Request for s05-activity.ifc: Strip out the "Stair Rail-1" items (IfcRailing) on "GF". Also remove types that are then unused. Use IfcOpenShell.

First a look at what the model holds.

```python
import ifcopenshell
import ifcopenshell.util.element

model = ifcopenshell.open("s05-activity.ifc")
print(model.schema)
storey = next(s for s in model.by_type("IfcBuildingStorey") if s.Name == "GF")
railings = [e for e in ifcopenshell.util.element.get_decomposition(storey) if e.is_a("IfcRailing")]
seen = {}
for e in railings:
    element_type = ifcopenshell.util.element.get_type(e)
    name = element_type.Name if element_type not in (None, e) else None
    seen[name] = seen.get(name, 0) + 1
for name, count in sorted(seen.items(), key=str):
    print(count, "x", name)
```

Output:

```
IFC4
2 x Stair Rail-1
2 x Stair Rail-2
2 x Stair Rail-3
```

```python
import ifcopenshell
import ifcopenshell.api.root
import ifcopenshell.util.element

model = ifcopenshell.open("s05-activity.ifc")

storey = next(s for s in model.by_type("IfcBuildingStorey") if s.Name == "GF")
railings = [e for e in ifcopenshell.util.element.get_decomposition(storey) if e.is_a("IfcRailing")]
targets = [e for e in railings if (t := ifcopenshell.util.element.get_type(e)) not in (None, e) and t.Name == "Stair Rail-1"]
types = {ifcopenshell.util.element.get_type(e) for e in targets} - {None, *targets}

for e in targets:
    ifcopenshell.api.root.remove_product(model, product=e)
print(len(targets), "removed")

unused = [t for t in types if not ifcopenshell.util.element.get_types(t)]
for t in unused:
    ifcopenshell.api.root.remove_product(model, product=t)
print(len(unused), "unused types removed")

model.write("s05-activity_edited.ifc")
```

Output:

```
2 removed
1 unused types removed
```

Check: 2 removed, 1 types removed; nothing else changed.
